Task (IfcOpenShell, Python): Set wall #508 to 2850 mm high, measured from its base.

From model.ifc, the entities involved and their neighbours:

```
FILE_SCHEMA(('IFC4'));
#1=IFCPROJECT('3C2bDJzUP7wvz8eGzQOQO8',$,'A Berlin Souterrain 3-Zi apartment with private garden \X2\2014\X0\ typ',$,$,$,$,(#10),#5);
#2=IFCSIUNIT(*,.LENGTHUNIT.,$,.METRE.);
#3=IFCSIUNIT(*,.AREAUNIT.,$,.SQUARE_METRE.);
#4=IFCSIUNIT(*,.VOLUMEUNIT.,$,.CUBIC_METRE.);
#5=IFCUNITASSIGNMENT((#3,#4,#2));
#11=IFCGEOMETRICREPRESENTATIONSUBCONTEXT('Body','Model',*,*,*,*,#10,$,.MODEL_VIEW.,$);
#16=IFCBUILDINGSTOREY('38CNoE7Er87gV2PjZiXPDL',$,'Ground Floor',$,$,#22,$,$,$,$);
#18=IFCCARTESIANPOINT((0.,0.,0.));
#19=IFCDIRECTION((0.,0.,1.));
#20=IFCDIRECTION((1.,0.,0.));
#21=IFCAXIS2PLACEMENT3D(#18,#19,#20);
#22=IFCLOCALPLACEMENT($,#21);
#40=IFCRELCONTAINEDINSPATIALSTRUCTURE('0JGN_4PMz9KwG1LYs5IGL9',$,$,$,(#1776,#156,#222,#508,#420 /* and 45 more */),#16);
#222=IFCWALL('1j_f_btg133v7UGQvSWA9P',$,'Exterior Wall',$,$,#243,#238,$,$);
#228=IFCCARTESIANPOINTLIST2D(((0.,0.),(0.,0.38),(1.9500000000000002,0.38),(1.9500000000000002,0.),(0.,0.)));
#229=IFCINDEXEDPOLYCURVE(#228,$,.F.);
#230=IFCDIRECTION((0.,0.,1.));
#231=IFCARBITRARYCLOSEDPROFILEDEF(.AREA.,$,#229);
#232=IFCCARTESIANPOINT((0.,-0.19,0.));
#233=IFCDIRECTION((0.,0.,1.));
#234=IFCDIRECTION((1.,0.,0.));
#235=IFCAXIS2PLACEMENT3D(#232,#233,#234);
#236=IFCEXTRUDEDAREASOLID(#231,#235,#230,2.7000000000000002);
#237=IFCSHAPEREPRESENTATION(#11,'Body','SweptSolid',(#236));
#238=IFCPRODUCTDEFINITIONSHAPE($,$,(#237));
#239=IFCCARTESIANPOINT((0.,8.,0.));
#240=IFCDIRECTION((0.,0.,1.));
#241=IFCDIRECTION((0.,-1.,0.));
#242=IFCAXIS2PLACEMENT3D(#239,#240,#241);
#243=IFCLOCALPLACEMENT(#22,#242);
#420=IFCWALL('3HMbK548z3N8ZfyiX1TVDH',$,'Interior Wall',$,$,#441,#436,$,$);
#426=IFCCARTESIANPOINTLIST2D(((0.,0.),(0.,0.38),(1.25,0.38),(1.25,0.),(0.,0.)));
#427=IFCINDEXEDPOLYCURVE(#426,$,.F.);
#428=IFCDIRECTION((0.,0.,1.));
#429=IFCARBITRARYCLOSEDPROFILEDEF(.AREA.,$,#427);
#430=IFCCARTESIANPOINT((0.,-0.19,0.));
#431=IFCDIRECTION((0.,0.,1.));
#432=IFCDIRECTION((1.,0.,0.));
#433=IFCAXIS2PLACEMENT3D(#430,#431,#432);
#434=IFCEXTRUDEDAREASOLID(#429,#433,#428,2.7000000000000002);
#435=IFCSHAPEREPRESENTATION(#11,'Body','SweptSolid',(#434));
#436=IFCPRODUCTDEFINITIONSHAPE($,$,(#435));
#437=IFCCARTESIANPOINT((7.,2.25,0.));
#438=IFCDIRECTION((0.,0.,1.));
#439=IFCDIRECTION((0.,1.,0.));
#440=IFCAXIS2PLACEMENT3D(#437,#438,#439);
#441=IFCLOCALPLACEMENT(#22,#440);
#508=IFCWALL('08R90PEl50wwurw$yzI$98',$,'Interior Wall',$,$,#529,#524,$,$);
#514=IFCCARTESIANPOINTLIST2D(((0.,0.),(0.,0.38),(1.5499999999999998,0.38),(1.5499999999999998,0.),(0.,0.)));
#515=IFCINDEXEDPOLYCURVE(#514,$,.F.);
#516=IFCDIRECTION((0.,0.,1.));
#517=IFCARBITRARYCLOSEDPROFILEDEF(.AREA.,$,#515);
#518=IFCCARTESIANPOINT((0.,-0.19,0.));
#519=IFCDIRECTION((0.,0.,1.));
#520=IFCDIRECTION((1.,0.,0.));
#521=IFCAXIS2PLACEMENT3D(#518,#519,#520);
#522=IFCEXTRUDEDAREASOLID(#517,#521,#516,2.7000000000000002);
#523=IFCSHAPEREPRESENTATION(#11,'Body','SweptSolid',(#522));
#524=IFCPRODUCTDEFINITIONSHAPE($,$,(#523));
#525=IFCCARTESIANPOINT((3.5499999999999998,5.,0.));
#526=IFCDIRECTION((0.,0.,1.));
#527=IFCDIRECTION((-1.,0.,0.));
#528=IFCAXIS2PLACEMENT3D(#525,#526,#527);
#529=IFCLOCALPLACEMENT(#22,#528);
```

```python
import ifcopenshell
import ifcopenshell.geom
import ifcopenshell.util.representation
import ifcopenshell.util.shape
import ifcopenshell.util.unit

model = ifcopenshell.open("model.ifc")
unit_scale = ifcopenshell.util.unit.calculate_unit_scale(model)
settings = ifcopenshell.geom.settings()


def volume(element):
    """Net volume in cubic metres, openings subtracted."""
    shape = ifcopenshell.geom.create_shape(settings, element)
    return ifcopenshell.util.shape.get_volume(shape.geometry)


wall = model.by_guid("08R90PEl50wwurw$yzI$98")
before = volume(wall)

body = ifcopenshell.util.representation.get_representation(wall, "Model", "Body")
solid = body.Items[0]
old_height = solid.Depth
solid.Depth = 2.85 / unit_scale
after = volume(wall)

print(f"height {old_height:g} -> {solid.Depth:g}, volume {before:.3f} -> {after:.3f} m3")

model.write("model_updated.ifc")
```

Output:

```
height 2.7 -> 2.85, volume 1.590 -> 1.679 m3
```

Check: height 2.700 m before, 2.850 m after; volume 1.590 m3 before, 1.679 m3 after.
